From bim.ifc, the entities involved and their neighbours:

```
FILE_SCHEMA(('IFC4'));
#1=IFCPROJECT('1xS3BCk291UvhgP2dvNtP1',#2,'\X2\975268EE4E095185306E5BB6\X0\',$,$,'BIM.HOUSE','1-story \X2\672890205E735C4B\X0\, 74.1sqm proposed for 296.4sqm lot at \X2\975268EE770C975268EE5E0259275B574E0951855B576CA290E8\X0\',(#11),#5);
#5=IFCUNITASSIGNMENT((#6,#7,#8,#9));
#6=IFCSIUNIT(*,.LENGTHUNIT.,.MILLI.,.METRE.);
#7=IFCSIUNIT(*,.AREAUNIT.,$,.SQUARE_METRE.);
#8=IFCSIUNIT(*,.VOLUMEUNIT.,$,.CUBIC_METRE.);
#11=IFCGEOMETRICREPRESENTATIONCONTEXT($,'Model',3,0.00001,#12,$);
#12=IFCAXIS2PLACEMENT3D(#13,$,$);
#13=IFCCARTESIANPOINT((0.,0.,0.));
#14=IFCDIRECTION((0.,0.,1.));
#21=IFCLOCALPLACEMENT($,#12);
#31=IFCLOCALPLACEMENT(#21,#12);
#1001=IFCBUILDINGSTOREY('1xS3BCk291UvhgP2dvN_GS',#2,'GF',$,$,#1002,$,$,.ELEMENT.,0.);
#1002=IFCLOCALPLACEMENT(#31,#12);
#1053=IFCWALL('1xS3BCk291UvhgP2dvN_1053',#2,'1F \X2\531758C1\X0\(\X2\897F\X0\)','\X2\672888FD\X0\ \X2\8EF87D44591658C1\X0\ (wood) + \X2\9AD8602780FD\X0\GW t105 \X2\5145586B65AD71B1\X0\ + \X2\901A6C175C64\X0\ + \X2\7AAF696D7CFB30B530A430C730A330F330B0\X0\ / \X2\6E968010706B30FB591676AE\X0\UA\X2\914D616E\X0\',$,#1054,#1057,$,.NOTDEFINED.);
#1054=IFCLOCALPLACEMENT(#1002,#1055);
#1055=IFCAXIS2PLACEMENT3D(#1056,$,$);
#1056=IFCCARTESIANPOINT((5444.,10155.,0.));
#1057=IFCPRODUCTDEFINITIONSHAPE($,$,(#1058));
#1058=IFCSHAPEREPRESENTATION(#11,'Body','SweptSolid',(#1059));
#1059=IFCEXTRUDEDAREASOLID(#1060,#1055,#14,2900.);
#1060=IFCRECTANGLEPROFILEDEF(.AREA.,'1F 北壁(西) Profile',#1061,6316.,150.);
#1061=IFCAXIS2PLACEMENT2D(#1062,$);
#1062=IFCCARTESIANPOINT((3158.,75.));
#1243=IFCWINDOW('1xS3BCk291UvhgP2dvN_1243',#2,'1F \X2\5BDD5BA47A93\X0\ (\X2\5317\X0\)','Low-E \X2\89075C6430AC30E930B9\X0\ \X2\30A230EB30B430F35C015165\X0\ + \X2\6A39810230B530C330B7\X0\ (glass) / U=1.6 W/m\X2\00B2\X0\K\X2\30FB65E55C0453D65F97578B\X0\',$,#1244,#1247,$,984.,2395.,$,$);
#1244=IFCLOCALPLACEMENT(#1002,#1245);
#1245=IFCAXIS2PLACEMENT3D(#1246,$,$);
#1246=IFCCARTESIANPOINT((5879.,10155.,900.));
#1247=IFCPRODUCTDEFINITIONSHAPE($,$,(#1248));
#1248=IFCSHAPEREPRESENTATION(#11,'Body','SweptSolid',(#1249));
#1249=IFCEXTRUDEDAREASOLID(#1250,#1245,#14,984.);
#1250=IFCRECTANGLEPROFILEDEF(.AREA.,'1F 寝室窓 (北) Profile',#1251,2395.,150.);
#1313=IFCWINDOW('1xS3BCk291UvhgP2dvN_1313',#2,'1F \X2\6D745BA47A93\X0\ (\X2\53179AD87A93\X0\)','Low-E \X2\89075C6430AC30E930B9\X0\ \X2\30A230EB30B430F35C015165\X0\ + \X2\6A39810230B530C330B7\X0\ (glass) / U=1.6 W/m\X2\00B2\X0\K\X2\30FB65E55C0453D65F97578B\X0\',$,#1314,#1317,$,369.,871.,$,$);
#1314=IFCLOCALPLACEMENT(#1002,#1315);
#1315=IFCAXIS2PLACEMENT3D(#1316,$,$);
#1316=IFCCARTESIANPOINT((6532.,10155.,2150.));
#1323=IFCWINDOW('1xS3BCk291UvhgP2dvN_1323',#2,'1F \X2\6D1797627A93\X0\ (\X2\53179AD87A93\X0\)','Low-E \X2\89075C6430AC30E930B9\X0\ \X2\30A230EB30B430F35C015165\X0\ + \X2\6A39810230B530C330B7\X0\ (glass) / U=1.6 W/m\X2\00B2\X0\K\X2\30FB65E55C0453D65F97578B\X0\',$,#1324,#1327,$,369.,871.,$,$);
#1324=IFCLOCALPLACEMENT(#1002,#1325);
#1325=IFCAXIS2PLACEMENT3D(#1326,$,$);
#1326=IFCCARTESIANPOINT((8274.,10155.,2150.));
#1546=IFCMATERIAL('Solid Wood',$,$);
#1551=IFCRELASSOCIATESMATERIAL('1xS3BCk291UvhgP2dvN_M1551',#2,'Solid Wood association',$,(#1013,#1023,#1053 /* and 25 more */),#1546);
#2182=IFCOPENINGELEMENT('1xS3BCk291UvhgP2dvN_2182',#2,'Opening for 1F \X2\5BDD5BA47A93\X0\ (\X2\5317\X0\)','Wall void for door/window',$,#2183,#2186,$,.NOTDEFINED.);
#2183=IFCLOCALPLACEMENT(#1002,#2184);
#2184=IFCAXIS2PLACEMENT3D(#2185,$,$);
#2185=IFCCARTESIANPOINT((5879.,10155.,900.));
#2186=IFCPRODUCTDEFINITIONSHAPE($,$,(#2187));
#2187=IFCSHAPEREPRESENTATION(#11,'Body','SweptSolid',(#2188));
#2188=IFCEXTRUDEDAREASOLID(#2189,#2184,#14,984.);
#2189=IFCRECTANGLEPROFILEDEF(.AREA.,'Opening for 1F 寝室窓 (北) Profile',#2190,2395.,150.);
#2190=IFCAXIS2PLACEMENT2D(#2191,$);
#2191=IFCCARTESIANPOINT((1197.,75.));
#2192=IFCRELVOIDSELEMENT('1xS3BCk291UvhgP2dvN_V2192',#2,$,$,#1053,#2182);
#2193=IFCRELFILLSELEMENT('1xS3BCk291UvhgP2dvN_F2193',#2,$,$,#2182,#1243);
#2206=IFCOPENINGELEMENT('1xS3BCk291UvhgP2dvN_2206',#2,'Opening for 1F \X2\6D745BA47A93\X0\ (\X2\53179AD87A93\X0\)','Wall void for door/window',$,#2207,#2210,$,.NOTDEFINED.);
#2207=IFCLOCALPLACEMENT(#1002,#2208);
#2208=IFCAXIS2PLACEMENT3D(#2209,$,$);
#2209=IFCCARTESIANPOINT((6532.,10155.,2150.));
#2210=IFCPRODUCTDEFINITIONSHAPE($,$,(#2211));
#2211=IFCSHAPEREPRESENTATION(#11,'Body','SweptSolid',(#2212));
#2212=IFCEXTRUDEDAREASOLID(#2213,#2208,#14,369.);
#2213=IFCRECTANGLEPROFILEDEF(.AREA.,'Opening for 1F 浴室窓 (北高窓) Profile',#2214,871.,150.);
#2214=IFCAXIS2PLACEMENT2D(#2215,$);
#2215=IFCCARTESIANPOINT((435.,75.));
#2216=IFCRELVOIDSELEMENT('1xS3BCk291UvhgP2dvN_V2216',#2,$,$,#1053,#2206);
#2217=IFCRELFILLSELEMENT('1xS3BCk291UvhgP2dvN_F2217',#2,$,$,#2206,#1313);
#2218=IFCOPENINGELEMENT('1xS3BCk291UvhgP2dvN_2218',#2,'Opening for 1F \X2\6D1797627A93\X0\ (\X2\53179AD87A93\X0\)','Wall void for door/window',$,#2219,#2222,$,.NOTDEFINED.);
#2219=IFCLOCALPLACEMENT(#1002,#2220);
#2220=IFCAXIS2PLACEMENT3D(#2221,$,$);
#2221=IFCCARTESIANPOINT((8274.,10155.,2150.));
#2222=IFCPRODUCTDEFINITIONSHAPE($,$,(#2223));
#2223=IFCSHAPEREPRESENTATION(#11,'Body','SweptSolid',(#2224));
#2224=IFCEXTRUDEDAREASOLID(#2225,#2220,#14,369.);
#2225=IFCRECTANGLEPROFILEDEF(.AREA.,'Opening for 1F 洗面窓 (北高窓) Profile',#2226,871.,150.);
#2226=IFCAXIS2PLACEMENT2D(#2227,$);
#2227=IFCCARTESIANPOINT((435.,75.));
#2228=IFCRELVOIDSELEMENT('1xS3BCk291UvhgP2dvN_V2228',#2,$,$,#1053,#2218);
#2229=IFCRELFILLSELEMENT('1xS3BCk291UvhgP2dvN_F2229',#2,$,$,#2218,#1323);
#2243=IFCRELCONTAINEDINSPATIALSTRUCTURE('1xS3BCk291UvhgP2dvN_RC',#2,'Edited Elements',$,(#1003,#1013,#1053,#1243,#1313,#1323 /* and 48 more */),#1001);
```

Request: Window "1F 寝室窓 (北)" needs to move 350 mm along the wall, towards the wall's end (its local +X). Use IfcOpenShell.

```python
import ifcopenshell
import ifcopenshell.api.geometry
import ifcopenshell.util.placement
import ifcopenshell.util.unit

model = ifcopenshell.open("bim.ifc")
unit_scale = ifcopenshell.util.unit.calculate_unit_scale(model)

window = model.by_guid("1xS3BCk291UvhgP2dvN_1243")
opening = window.FillsVoids[0].RelatingOpeningElement
wall = opening.VoidsElements[0].RelatingBuildingElement

wall_matrix = ifcopenshell.util.placement.get_local_placement(wall.ObjectPlacement)
shift = wall_matrix[:3, 0] * 0.35 / unit_scale
before = ifcopenshell.util.placement.get_local_placement(window.ObjectPlacement)[:3, 3].copy()

# The window is not placed relative to its opening, so move both.
for product in (opening, window):
    matrix = ifcopenshell.util.placement.get_local_placement(product.ObjectPlacement)
    matrix[:3, 3] += shift
    ifcopenshell.api.geometry.edit_object_placement(model, product=product, matrix=matrix, is_si=False)

after = ifcopenshell.util.placement.get_local_placement(window.ObjectPlacement)[:3, 3]
print("window moved by", (after - before).round(3) + 0.0)

model.write("bim_rev.ifc")
```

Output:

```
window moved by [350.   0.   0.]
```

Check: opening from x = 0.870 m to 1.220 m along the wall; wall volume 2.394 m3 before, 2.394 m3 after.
